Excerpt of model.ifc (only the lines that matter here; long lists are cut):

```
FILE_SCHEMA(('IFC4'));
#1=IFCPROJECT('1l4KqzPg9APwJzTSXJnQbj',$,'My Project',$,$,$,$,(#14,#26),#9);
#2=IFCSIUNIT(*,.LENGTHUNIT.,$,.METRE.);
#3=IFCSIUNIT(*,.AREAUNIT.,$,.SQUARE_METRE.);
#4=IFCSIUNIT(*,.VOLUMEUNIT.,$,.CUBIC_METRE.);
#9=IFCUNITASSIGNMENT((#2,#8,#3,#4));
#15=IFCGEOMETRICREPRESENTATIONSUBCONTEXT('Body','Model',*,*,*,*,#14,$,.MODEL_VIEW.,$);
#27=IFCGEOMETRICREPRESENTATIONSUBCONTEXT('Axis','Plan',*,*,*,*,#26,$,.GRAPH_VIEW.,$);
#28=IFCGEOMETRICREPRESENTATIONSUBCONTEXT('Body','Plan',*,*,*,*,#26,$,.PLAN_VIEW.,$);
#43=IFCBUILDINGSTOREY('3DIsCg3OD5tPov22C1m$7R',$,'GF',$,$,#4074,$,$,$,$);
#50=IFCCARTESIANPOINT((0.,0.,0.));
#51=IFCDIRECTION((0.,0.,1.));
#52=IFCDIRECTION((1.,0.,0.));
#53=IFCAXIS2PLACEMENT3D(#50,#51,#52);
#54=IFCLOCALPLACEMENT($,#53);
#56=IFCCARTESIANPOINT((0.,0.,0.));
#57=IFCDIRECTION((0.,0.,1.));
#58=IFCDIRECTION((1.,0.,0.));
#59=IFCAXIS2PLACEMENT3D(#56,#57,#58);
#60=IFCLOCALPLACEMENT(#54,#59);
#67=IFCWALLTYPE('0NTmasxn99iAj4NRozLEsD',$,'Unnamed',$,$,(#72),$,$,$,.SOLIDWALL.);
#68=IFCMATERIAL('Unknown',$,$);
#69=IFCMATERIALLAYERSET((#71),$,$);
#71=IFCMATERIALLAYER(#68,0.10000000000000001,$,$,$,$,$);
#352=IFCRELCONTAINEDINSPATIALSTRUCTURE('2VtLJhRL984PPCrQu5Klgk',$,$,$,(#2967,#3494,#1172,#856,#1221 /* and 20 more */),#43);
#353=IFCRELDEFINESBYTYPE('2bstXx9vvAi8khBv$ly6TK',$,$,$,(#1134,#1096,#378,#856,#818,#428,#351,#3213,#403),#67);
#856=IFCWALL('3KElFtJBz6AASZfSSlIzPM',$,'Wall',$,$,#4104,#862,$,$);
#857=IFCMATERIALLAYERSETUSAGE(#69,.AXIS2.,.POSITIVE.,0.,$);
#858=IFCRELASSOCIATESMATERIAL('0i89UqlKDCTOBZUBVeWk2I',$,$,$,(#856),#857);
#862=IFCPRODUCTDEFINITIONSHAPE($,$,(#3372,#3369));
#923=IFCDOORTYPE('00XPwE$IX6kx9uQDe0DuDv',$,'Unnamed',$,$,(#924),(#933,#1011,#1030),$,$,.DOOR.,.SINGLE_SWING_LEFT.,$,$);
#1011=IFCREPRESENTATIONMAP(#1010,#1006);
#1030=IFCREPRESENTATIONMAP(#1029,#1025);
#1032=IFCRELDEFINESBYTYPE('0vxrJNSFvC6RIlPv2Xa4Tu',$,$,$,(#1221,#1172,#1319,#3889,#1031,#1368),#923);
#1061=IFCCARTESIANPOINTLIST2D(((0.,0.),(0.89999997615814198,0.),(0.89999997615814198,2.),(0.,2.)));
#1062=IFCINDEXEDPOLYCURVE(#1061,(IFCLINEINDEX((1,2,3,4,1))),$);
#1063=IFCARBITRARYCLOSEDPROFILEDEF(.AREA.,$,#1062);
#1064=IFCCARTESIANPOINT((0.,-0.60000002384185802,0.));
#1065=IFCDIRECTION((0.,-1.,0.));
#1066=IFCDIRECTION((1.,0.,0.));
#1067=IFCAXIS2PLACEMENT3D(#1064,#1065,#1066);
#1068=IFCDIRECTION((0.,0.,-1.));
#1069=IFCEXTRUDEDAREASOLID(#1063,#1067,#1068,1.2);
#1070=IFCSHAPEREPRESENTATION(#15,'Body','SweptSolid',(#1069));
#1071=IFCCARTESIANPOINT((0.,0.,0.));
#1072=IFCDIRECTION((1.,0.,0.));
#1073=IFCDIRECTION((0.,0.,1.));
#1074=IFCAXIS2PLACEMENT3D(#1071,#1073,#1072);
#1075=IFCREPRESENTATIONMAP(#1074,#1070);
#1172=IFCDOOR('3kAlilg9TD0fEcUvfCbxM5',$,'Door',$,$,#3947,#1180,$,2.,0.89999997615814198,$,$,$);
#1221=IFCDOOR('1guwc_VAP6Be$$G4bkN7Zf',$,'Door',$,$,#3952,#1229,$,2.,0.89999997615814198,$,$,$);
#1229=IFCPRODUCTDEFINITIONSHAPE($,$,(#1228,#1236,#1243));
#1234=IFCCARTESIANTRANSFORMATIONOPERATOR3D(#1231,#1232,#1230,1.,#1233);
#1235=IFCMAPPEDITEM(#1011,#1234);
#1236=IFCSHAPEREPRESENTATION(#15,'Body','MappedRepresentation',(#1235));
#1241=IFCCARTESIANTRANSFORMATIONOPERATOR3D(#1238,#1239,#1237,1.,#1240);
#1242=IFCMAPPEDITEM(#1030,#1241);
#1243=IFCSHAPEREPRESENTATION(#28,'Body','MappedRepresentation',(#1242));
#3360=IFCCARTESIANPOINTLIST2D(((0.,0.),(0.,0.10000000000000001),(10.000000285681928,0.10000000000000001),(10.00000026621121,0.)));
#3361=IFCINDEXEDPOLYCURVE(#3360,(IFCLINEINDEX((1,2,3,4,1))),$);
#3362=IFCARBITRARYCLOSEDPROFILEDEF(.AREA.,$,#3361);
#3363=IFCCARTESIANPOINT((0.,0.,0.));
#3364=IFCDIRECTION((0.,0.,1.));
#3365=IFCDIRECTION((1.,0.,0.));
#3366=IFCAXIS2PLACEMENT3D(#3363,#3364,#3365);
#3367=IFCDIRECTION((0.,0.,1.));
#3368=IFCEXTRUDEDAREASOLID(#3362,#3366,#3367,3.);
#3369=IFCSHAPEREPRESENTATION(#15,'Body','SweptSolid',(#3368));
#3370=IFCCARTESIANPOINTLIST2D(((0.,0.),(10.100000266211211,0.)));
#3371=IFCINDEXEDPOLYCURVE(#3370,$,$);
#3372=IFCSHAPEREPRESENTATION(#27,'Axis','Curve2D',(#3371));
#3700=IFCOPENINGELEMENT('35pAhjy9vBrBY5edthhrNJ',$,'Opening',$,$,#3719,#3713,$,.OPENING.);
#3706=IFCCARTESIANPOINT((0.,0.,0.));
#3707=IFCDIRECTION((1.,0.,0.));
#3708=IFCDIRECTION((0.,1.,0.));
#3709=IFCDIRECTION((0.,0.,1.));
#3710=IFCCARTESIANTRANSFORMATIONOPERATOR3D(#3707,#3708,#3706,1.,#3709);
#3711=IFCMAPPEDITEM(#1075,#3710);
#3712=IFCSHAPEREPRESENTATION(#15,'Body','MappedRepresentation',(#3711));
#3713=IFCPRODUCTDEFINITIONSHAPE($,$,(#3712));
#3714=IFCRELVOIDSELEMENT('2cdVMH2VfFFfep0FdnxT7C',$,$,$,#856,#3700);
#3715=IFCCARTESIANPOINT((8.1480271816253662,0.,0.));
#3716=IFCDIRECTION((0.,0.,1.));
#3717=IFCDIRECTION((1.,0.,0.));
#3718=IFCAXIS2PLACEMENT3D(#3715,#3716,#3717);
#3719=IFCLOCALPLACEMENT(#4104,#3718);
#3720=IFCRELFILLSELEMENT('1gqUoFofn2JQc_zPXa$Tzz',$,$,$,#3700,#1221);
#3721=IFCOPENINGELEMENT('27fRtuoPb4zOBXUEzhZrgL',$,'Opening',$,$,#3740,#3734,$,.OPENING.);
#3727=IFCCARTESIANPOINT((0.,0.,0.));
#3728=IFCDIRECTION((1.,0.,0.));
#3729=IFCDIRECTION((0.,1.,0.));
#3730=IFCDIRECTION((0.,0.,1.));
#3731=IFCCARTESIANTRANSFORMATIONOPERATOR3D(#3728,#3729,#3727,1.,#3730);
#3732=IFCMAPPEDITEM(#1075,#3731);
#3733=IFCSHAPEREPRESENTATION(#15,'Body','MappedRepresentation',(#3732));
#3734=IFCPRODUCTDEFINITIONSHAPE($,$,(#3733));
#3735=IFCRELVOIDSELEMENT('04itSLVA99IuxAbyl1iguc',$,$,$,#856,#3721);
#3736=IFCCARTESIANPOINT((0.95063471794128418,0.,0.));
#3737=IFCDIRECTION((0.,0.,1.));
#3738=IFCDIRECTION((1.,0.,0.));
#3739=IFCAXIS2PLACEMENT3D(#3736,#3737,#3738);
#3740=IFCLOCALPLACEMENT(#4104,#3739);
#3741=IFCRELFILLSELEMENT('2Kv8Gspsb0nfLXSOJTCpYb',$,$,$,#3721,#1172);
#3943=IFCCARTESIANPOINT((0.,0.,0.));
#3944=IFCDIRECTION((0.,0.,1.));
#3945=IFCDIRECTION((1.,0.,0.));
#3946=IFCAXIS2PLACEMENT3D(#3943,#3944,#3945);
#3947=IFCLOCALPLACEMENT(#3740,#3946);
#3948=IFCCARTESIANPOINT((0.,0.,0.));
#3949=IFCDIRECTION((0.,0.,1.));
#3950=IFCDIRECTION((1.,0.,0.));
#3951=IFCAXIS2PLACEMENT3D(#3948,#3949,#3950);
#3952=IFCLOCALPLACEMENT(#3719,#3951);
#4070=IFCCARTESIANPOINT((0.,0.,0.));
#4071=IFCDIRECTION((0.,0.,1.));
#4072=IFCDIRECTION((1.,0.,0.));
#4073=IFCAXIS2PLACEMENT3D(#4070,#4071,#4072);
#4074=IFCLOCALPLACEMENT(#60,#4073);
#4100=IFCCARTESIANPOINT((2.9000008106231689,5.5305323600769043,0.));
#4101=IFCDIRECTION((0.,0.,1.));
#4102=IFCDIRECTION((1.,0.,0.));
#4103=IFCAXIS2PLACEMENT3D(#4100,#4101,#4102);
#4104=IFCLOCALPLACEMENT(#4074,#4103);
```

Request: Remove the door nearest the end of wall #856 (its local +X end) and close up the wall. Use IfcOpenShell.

```python
import ifcopenshell
import ifcopenshell.api.feature
import ifcopenshell.api.root
import ifcopenshell.geom
import ifcopenshell.util.shape

model = ifcopenshell.open("model.ifc")
settings = ifcopenshell.geom.settings()


def volume(element):
    """Net volume in cubic metres, openings subtracted."""
    shape = ifcopenshell.geom.create_shape(settings, element)
    return ifcopenshell.util.shape.get_volume(shape.geometry)


door = model.by_guid("1guwc_VAP6Be$$G4bkN7Zf")
opening = door.FillsVoids[0].RelatingOpeningElement
wall = opening.VoidsElements[0].RelatingBuildingElement
before = volume(wall)

ifcopenshell.api.root.remove_product(model, product=door)
ifcopenshell.api.feature.remove_feature(model, feature=opening)

after = volume(wall)

print(f"wall volume {before:.3f} -> {after:.3f} m3")

model.write("model_rev.ifc")
```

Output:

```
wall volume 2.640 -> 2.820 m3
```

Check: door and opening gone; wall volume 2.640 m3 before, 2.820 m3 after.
